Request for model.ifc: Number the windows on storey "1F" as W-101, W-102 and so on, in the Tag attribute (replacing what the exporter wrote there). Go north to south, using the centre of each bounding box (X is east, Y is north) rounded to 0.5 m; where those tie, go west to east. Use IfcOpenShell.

First a look at what the model holds.

```python
import ifcopenshell
import ifcopenshell.util.element
import ifcopenshell.util.placement

model = ifcopenshell.open("model.ifc")
print(model.schema)
storey = next(s for s in model.by_type("IfcBuildingStorey") if s.Name == "1F")
windows = [e for e in ifcopenshell.util.element.get_decomposition(storey) if e.is_a("IfcWindow")]
for e in sorted(windows, key=lambda e: e.id()):
    origin = ifcopenshell.util.placement.get_local_placement(e.ObjectPlacement)[:3, 3]
    print(e.id(), e.Tag, e.Name, origin.round(2) + 0.0, sep=" | ")
```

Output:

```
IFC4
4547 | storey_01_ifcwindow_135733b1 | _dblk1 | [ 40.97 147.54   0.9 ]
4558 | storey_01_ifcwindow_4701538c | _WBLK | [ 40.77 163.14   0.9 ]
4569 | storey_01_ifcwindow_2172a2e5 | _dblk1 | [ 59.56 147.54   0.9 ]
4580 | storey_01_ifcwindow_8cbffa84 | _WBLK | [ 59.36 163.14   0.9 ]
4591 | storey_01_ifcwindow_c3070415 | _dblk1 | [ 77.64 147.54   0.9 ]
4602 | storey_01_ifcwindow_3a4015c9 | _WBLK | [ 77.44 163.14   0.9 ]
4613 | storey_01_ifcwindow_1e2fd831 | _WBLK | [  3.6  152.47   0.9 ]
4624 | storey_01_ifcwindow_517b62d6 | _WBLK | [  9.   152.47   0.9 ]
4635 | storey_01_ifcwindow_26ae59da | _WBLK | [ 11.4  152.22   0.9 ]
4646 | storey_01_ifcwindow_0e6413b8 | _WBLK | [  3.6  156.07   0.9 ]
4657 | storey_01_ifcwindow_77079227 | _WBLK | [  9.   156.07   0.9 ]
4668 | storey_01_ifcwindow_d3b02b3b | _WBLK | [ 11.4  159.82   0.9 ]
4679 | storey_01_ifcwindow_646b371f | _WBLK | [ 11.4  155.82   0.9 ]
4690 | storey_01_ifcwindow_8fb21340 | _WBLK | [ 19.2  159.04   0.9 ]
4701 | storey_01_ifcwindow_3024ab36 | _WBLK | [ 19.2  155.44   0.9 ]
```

```python
import ifcopenshell
import ifcopenshell.geom
import ifcopenshell.util.element
import ifcopenshell.util.shape

model = ifcopenshell.open("model.ifc")
settings = ifcopenshell.geom.settings()
settings.set("use-world-coords", True)


def centre(element):
    shape = ifcopenshell.geom.create_shape(settings, element)
    return ifcopenshell.util.shape.get_bbox_centroid(shape.geometry)


storey = next(s for s in model.by_type("IfcBuildingStorey") if s.Name == "1F")
windows = [e for e in ifcopenshell.util.element.get_decomposition(storey) if e.is_a("IfcWindow")]

# Insertion points can sit at a corner or the storey origin, so sort by the geometry (in metres).
centres = {e: centre(e) for e in windows}
windows.sort(key=lambda e: (-round(centres[e][1] / 0.5), centres[e][0]))

for i, e in enumerate(windows, start=1):
    number = f"W-1{i:02d}"
    e.Tag = number
    print(e.id(), number)

model.write("model_v2.ifc")
```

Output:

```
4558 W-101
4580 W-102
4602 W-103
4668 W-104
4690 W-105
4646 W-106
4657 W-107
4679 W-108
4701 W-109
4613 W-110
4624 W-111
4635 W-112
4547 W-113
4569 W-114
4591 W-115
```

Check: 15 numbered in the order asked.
